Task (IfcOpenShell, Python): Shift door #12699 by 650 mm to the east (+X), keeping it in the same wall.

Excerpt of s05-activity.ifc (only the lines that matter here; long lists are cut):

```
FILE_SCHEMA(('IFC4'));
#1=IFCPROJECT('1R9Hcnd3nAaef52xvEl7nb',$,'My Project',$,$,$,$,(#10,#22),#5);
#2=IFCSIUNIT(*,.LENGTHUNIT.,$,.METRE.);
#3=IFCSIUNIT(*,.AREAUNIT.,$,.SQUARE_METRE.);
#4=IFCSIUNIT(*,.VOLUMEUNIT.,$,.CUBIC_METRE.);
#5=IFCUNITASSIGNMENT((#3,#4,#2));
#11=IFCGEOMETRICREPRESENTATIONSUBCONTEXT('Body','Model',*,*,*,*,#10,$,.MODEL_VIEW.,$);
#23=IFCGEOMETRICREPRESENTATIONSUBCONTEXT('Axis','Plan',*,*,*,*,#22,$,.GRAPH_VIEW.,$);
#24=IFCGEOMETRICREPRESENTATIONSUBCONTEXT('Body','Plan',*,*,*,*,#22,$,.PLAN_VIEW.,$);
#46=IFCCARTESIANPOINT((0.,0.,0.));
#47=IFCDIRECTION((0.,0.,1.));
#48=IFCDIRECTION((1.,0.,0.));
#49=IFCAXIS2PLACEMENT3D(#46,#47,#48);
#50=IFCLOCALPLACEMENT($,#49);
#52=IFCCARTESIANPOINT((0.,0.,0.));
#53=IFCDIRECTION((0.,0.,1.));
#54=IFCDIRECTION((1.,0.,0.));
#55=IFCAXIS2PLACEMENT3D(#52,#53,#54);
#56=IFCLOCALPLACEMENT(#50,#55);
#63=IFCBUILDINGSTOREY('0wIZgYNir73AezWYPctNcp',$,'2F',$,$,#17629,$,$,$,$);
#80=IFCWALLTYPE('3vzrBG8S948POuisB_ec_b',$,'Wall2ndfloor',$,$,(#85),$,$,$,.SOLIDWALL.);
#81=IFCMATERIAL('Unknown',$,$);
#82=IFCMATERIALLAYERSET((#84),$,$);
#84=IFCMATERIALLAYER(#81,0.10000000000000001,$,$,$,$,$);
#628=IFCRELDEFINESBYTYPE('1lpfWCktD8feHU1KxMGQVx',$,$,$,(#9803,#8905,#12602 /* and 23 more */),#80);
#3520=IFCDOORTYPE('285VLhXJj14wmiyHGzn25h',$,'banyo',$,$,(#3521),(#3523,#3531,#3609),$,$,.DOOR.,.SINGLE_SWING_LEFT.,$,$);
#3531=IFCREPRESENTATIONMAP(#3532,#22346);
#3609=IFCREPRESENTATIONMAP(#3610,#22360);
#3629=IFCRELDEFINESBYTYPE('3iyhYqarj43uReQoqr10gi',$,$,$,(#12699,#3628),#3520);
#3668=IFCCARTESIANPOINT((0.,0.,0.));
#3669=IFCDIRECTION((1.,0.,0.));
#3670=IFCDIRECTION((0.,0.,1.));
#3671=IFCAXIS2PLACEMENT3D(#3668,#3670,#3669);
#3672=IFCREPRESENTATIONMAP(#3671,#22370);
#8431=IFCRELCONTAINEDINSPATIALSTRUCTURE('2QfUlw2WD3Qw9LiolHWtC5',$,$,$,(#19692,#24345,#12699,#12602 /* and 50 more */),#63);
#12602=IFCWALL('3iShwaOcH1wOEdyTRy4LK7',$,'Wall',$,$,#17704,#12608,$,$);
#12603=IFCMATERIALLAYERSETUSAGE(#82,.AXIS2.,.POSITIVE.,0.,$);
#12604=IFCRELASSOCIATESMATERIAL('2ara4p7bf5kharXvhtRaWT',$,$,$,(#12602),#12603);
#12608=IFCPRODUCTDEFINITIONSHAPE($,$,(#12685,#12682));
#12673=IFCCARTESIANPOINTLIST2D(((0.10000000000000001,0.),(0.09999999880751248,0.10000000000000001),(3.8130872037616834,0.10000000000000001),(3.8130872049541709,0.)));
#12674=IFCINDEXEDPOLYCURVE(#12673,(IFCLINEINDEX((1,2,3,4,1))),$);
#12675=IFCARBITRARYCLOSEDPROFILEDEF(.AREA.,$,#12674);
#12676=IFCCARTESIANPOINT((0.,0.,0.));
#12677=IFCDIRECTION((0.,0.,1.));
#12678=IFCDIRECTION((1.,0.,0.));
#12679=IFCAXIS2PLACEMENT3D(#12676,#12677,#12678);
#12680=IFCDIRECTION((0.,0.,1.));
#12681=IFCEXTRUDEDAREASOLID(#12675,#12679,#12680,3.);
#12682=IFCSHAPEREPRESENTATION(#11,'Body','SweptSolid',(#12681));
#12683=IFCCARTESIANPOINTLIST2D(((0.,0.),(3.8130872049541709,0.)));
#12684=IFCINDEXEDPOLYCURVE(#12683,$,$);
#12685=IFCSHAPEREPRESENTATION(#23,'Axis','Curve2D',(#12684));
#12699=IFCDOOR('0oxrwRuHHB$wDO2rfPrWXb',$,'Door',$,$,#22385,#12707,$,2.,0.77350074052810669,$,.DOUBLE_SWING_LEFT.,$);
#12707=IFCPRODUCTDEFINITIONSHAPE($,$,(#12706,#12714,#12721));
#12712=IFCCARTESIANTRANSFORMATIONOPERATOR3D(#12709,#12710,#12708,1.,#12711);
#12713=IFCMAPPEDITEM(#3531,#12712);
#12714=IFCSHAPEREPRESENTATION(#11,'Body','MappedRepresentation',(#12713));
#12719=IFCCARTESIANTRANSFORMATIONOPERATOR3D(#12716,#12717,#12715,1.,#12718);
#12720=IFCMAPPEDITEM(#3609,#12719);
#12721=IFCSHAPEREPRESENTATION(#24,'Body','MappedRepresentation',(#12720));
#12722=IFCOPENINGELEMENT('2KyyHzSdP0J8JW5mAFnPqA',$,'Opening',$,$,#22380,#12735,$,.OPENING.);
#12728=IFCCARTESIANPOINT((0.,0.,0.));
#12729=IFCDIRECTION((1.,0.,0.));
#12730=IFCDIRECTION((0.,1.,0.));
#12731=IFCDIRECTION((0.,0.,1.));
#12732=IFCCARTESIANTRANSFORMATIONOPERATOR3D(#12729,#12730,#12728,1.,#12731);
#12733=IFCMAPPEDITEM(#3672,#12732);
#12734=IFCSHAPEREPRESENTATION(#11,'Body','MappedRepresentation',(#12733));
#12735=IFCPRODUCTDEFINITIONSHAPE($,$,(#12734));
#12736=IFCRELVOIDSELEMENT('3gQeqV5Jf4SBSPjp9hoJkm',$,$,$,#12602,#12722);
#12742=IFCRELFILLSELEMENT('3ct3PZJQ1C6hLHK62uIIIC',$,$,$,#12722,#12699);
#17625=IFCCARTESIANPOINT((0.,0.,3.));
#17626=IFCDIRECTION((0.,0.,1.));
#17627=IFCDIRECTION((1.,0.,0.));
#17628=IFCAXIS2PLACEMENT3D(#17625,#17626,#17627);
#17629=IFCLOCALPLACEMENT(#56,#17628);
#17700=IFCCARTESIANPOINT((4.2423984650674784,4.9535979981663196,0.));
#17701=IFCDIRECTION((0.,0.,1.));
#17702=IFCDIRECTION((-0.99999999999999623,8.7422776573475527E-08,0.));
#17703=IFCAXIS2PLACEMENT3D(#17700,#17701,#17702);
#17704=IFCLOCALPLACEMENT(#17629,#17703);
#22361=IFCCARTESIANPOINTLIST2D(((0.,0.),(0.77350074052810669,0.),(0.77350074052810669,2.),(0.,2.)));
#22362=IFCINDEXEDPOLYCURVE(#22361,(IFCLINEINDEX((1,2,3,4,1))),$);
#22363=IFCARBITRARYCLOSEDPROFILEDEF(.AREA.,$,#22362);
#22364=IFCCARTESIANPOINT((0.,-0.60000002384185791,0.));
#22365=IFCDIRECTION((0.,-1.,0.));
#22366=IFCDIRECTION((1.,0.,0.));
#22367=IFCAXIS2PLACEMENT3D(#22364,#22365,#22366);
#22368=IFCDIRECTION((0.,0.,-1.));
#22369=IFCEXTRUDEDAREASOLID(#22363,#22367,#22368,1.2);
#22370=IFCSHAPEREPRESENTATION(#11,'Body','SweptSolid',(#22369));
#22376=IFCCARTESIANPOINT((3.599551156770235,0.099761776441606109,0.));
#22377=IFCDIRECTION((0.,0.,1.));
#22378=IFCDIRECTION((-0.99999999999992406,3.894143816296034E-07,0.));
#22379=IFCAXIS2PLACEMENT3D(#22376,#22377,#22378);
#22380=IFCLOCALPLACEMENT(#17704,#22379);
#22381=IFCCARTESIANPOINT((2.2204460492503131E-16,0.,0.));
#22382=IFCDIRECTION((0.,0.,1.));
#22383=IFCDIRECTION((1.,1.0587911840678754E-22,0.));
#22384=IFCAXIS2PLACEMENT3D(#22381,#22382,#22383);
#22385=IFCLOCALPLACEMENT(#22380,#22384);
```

```python
import ifcopenshell
import ifcopenshell.api.geometry
import ifcopenshell.util.placement

model = ifcopenshell.open("s05-activity.ifc")

door = model.by_guid("0oxrwRuHHB$wDO2rfPrWXb")
opening = door.FillsVoids[0].RelatingOpeningElement
wall = opening.VoidsElements[0].RelatingBuildingElement

wall_matrix = ifcopenshell.util.placement.get_local_placement(wall.ObjectPlacement)
shift = wall_matrix[:3, 0] * -0.65
before = ifcopenshell.util.placement.get_local_placement(door.ObjectPlacement)[:3, 3].copy()

# The door is placed relative to its opening, so it follows when the opening moves.
matrix = ifcopenshell.util.placement.get_local_placement(opening.ObjectPlacement)
matrix[:3, 3] += shift
ifcopenshell.api.geometry.edit_object_placement(
    model, product=opening, matrix=matrix, is_si=False, should_transform_children=True
)

after = ifcopenshell.util.placement.get_local_placement(door.ObjectPlacement)[:3, 3]
print("door moved by", (after - before).round(3) + 0.0)

model.write("s05-activity_rev.ifc")
```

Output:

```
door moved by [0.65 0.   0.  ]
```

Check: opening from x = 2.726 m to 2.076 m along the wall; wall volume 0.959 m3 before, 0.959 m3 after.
